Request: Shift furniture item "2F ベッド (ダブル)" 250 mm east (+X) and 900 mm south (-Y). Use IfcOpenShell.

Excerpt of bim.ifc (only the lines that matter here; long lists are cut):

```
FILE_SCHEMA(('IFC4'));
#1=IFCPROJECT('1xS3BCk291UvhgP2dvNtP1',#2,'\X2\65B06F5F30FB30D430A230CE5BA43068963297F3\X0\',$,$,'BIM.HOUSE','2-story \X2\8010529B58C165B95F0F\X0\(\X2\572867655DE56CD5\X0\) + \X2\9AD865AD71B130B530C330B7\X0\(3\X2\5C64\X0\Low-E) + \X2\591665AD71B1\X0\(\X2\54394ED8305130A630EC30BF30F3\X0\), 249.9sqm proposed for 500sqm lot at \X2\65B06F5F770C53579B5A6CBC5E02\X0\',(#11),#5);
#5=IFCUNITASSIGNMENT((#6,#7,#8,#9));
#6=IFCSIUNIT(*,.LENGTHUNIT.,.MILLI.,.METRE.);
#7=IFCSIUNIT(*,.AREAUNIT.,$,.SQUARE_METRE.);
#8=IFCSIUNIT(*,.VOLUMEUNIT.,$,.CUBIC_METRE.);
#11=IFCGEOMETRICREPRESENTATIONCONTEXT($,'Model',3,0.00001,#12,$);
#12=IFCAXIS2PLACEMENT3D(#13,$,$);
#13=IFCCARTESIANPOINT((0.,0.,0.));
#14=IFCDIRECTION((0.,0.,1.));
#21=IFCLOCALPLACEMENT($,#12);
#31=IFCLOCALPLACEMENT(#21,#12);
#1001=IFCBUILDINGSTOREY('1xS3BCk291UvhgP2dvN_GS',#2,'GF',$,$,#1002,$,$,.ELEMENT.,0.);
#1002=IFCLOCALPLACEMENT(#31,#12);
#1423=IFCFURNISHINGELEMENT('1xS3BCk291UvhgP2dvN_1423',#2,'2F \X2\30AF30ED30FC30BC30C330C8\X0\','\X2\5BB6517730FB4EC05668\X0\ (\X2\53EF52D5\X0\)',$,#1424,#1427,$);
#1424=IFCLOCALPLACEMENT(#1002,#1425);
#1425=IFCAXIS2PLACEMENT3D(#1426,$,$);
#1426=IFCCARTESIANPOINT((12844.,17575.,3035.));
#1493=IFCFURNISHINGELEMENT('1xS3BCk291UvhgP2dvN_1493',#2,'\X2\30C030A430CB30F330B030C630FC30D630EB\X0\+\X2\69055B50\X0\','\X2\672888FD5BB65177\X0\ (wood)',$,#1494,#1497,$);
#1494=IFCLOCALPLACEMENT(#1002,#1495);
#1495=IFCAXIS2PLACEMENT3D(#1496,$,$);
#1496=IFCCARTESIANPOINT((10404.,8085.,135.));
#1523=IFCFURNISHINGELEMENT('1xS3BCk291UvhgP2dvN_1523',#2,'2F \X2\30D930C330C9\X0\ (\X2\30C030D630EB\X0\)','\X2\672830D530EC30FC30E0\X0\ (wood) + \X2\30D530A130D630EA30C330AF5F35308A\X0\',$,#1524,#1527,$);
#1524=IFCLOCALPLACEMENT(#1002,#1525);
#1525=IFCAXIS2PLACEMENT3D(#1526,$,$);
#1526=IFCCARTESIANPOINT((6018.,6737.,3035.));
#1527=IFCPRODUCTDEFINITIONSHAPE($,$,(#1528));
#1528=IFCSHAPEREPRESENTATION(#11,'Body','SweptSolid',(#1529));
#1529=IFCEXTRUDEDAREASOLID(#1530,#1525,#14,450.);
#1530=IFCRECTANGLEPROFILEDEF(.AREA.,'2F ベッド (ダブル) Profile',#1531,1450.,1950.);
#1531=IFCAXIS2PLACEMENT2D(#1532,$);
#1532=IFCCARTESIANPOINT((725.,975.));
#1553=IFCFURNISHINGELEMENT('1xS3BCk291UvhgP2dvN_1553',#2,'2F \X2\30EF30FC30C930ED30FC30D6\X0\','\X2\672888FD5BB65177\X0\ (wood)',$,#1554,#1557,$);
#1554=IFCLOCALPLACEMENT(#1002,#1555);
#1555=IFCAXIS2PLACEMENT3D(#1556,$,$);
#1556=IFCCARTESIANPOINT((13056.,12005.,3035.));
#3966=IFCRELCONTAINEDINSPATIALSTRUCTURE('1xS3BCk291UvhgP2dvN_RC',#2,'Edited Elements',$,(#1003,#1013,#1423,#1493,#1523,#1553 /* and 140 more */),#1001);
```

```python
import ifcopenshell
import ifcopenshell.api.geometry
import ifcopenshell.util.placement

model = ifcopenshell.open("bim.ifc")

item = model.by_guid("1xS3BCk291UvhgP2dvN_1523")
matrix = ifcopenshell.util.placement.get_local_placement(item.ObjectPlacement)
matrix[0, 3] += 250.0
matrix[1, 3] -= 900.0
ifcopenshell.api.geometry.edit_object_placement(model, product=item, matrix=matrix, is_si=False)

print(ifcopenshell.util.placement.get_local_placement(item.ObjectPlacement).round(3) + 0.0)

model.write("bim_edited.ifc")
```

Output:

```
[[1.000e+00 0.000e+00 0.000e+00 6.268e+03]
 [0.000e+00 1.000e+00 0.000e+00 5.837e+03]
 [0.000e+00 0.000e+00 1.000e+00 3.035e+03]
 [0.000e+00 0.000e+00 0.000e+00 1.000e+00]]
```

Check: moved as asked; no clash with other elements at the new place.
